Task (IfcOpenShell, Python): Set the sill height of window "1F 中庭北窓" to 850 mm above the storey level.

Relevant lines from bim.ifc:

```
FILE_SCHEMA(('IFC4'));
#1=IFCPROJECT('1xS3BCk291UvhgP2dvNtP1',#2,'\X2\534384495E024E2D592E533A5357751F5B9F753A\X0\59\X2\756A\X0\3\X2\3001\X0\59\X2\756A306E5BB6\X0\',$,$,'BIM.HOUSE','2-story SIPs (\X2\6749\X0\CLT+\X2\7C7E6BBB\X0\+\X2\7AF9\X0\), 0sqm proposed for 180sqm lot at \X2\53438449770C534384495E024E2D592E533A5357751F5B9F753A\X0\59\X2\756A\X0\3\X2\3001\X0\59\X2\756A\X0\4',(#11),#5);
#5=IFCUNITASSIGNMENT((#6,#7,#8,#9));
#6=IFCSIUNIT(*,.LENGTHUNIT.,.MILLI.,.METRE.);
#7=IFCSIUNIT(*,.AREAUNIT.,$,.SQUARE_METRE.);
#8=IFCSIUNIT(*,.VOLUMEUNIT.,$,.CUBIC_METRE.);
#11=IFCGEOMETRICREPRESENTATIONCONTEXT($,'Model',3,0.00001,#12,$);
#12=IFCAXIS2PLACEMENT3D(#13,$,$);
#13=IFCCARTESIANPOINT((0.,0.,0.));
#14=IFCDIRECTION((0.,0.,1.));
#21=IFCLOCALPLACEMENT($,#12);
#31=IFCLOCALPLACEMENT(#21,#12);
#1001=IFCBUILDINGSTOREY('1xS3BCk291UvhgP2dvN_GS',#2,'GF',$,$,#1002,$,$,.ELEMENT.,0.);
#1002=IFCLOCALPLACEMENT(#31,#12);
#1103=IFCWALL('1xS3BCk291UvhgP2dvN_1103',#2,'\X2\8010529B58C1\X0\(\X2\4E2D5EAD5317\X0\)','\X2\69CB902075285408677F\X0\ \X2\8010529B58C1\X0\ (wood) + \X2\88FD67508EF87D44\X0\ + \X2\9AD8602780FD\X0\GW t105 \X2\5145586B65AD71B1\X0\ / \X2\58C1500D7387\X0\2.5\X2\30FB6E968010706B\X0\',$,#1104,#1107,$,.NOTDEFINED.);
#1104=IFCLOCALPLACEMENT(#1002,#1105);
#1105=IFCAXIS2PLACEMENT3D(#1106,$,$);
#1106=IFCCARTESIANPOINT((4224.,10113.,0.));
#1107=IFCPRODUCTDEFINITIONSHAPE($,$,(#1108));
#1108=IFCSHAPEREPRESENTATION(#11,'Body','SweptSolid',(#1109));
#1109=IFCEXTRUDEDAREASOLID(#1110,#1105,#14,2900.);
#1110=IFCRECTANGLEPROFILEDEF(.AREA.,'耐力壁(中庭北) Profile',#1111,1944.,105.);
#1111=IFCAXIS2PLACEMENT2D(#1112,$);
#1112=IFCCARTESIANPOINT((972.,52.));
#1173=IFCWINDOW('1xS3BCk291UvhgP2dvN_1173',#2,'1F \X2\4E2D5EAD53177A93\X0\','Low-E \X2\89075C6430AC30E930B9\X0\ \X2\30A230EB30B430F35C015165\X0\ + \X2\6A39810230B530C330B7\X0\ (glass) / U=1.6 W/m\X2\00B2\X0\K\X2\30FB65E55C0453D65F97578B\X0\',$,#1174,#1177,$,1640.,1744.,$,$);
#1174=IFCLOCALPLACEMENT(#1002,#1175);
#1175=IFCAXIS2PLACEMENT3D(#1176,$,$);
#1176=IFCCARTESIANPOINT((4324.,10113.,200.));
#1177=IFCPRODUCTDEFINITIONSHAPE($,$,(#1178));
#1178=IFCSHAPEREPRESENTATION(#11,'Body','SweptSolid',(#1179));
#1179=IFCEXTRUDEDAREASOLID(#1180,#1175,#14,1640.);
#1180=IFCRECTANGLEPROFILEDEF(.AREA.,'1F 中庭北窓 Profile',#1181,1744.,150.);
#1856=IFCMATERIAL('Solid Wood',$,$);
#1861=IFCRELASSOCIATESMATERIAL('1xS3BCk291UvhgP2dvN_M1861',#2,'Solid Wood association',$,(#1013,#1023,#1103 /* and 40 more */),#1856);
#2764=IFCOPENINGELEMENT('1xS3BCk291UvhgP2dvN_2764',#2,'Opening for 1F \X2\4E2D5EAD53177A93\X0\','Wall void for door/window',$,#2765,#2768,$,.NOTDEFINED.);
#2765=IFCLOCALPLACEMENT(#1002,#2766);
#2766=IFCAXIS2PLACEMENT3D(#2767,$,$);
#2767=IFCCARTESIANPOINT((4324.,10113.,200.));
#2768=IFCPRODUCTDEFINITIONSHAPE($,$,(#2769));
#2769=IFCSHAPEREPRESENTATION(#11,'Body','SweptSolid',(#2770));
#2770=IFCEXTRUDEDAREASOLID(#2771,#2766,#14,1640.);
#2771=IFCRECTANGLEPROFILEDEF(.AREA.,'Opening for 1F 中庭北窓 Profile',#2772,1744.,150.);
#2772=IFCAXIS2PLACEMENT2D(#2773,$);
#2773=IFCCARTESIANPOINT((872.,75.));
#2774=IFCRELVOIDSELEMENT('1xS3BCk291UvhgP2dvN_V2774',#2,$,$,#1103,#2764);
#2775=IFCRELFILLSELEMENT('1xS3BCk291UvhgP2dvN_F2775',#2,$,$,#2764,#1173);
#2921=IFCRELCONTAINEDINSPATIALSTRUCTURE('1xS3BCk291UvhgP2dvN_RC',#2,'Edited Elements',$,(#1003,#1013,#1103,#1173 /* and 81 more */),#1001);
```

```python
import numpy as np
import ifcopenshell
import ifcopenshell.api.geometry
import ifcopenshell.geom
import ifcopenshell.util.element
import ifcopenshell.util.placement
import ifcopenshell.util.shape
import ifcopenshell.util.unit

model = ifcopenshell.open("bim.ifc")
unit_scale = ifcopenshell.util.unit.calculate_unit_scale(model)

window = model.by_id(1173)
opening = window.FillsVoids[0].RelatingOpeningElement
storey = ifcopenshell.util.element.get_container(window, ifc_class="IfcBuildingStorey")
level = ifcopenshell.util.placement.get_local_placement(storey.ObjectPlacement)[2, 3]

# The opening's origin need not be at the sill, so measure its lowest point.
shape = ifcopenshell.geom.create_shape(ifcopenshell.geom.settings(), opening)
bottom = ifcopenshell.util.shape.get_shape_bottom_elevation(shape, shape.geometry) / unit_scale
dz = level + 0.85 / unit_scale - bottom

shift = np.array([0.0, 0.0, dz])
# The window is not placed relative to its opening, so move both.
for product in (opening, window):
    matrix = ifcopenshell.util.placement.get_local_placement(product.ObjectPlacement)
    matrix[:3, 3] += shift
    ifcopenshell.api.geometry.edit_object_placement(model, product=product, matrix=matrix, is_si=False)

print(f"moved by {dz * unit_scale:+.3f} m")

model.write("bim_v2.ifc")
```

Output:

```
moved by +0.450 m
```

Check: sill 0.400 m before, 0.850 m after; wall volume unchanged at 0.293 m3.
